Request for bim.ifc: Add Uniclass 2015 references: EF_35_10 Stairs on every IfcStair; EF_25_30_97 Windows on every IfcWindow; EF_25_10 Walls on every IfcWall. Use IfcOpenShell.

First a look at what the model holds.

```python
import ifcopenshell

model = ifcopenshell.open("bim.ifc")
print(model.schema)
print("classifications:", [c.Name for c in model.by_type("IfcClassification")])
for ifc_class in ("IfcDoor", "IfcRoof", "IfcStair", "IfcWall", "IfcWindow"):
    print(ifc_class, len(model.by_type(ifc_class)))
```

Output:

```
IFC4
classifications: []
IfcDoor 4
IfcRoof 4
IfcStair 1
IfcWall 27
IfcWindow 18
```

```python
import ifcopenshell
import ifcopenshell.api.classification

model = ifcopenshell.open("bim.ifc")

system = ifcopenshell.api.classification.add_classification(model, classification="Uniclass 2015")

codes = {
    "IfcStair": ("EF_35_10", "Stairs"),
    "IfcWindow": ("EF_25_30_97", "Windows"),
    "IfcWall": ("EF_25_10", "Walls"),
}
for ifc_class, (code, name) in codes.items():
    products = model.by_type(ifc_class)
    ifcopenshell.api.classification.add_reference(
        model, products=products, classification=system, identification=code, name=name
    )
    print(code, len(products))

model.write("bim_v2.ifc")
```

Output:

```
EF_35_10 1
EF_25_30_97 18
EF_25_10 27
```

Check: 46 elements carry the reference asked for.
